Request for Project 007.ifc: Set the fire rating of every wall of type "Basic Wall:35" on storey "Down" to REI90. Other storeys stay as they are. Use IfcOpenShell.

First a look at what the model holds.

```python
import ifcopenshell
import ifcopenshell.util.element

model = ifcopenshell.open("Project 007.ifc")
print(model.schema)
storey = next(s for s in model.by_type("IfcBuildingStorey") if s.Name == "Down")
walls = [e for e in ifcopenshell.util.element.get_decomposition(storey) if e.is_a("IfcWall")]
seen = {}
for e in walls:
    element_type = ifcopenshell.util.element.get_type(e)
    key = (element_type.Name if element_type != e and element_type else None, ifcopenshell.util.element.get_pset(e, "Pset_WallCommon", "FireRating"))
    seen[key] = seen.get(key, 0) + 1
for (name, value), count in sorted(seen.items(), key=str):
    print(count, "x", name, "|", value)
```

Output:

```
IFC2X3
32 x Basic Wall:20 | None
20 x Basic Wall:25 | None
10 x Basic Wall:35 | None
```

```python
import ifcopenshell
import ifcopenshell.api.pset
import ifcopenshell.util.element

model = ifcopenshell.open("Project 007.ifc")

storey = next(s for s in model.by_type("IfcBuildingStorey") if s.Name == "Down")
walls = [e for e in ifcopenshell.util.element.get_decomposition(storey) if e.is_a("IfcWall")]

count = 0
for e in walls:
    element_type = ifcopenshell.util.element.get_type(e)
    if element_type in (None, e) or element_type.Name != "Basic Wall:35":
        continue
    # add_pset returns the element's existing set when there is one.
    pset = ifcopenshell.api.pset.add_pset(model, product=e, name="Pset_WallCommon")
    ifcopenshell.api.pset.edit_pset(model, pset=pset, properties={"FireRating": "REI90"})
    count += 1

print(count, "walls updated")

model.write("Project 007_v2.ifc")
```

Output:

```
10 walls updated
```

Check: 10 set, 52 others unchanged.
